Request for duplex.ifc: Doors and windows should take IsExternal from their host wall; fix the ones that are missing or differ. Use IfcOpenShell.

First a look at what the model holds.

```python
import ifcopenshell
import ifcopenshell.util.element

model = ifcopenshell.open("duplex.ifc")
print(model.schema)
seen = {}
for e in model.by_type("IfcDoor") + model.by_type("IfcWindow"):
    if not e.FillsVoids:
        continue
    host = e.FillsVoids[0].RelatingOpeningElement.VoidsElements[0].RelatingBuildingElement
    own = ifcopenshell.util.element.get_pset(e, f"Pset_{e.is_a()[3:].removesuffix('StandardCase')}Common", "IsExternal")
    wall = ifcopenshell.util.element.get_pset(host, "Pset_WallCommon", "IsExternal")
    seen[e.is_a(), own, wall] = seen.get((e.is_a(), own, wall), 0) + 1
for (cls, own, wall), count in sorted(seen.items(), key=str):
    print(count, cls, "IsExternal:", own, "| host wall:", wall)
```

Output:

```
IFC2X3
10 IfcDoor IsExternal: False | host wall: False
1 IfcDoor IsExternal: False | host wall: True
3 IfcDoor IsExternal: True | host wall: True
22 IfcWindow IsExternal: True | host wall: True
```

```python
import ifcopenshell
import ifcopenshell.api.pset
import ifcopenshell.util.element

model = ifcopenshell.open("duplex.ifc")

count = 0
for ifc_class, pset_name in (("IfcDoor", "Pset_DoorCommon"), ("IfcWindow", "Pset_WindowCommon")):
    for e in model.by_type(ifc_class):
        if not e.FillsVoids:
            continue
        host = e.FillsVoids[0].RelatingOpeningElement.VoidsElements[0].RelatingBuildingElement
        external = ifcopenshell.util.element.get_pset(host, "Pset_WallCommon", "IsExternal")
        if external is None or ifcopenshell.util.element.get_pset(e, pset_name, "IsExternal") == external:
            continue
        pset = ifcopenshell.api.pset.add_pset(model, product=e, name=pset_name)
        ifcopenshell.api.pset.edit_pset(model, pset=pset, properties={"IsExternal": external})
        count += 1

print(count, "updated")

model.write("duplex_updated.ifc")
```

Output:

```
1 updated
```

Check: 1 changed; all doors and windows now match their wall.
